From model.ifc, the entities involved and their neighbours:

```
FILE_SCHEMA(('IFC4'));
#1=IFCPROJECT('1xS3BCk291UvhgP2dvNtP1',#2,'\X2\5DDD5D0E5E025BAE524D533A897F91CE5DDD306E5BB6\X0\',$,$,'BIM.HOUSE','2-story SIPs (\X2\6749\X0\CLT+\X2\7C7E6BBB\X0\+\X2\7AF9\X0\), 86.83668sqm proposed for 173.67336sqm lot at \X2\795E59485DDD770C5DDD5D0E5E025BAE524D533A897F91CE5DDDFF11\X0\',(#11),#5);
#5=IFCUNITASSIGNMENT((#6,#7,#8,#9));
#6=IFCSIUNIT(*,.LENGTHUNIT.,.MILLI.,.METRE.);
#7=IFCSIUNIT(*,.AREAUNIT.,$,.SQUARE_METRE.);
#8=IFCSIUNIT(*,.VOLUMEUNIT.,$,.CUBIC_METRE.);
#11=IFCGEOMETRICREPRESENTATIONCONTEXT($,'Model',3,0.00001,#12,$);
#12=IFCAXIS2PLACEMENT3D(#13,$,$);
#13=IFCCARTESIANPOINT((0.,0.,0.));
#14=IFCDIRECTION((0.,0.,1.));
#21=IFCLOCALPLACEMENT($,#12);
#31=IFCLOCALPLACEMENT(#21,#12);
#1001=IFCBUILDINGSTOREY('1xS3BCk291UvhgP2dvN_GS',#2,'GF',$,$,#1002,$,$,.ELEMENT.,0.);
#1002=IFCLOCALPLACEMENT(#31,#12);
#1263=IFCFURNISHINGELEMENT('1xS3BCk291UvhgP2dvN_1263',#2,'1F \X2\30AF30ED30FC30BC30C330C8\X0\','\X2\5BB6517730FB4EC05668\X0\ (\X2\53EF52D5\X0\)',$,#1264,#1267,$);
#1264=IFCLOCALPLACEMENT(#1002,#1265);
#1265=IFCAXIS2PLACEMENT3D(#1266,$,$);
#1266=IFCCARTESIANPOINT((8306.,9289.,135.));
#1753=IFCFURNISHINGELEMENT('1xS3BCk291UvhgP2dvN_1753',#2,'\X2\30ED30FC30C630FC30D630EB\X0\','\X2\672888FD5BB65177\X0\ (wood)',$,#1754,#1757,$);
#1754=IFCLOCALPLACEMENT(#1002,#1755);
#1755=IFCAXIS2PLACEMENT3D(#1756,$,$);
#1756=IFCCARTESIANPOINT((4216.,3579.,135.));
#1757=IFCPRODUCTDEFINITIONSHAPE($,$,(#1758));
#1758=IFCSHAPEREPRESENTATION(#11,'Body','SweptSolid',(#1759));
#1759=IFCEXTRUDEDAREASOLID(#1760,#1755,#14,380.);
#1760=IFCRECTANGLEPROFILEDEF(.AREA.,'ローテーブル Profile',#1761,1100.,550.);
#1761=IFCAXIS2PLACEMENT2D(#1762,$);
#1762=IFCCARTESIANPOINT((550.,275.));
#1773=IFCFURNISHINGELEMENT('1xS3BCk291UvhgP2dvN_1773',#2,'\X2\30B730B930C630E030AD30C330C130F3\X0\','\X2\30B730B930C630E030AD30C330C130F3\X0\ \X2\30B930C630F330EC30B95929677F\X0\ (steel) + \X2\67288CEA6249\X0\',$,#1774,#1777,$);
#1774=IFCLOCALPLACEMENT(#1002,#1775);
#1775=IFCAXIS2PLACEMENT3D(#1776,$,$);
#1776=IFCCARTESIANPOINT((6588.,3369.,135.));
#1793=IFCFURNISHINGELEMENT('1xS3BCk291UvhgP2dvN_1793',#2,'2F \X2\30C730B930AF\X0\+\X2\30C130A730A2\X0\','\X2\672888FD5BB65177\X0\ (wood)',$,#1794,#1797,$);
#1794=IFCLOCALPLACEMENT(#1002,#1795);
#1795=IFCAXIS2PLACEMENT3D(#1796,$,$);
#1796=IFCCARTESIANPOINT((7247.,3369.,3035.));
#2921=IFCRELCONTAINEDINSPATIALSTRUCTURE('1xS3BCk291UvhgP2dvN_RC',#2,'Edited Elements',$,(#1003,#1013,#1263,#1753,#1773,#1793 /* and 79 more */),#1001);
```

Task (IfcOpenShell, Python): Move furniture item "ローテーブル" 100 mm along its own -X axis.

```python
import ifcopenshell
import ifcopenshell.api.geometry
import ifcopenshell.util.placement
import ifcopenshell.util.unit

model = ifcopenshell.open("model.ifc")
unit_scale = ifcopenshell.util.unit.calculate_unit_scale(model)

item = model.by_guid("1xS3BCk291UvhgP2dvN_1753")
matrix = ifcopenshell.util.placement.get_local_placement(item.ObjectPlacement)
matrix[:3, 3] -= matrix[:3, 0] * 0.1 / unit_scale
ifcopenshell.api.geometry.edit_object_placement(model, product=item, matrix=matrix, is_si=False)

print(ifcopenshell.util.placement.get_local_placement(item.ObjectPlacement).round(3) + 0.0)

model.write("model_rev.ifc")
```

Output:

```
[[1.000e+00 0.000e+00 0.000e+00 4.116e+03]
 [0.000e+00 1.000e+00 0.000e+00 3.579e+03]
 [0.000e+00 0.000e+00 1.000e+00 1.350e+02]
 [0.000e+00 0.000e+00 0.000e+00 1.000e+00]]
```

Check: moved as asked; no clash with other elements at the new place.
